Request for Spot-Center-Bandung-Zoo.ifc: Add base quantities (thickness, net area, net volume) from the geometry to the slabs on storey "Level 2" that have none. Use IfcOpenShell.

First a look at what the model holds.

```python
import ifcopenshell
import ifcopenshell.util.element
import ifcopenshell.util.unit

model = ifcopenshell.open("Spot-Center-Bandung-Zoo.ifc")
print(model.schema)
for unit_type in ("LENGTHUNIT", "AREAUNIT", "VOLUMEUNIT"):
    print(unit_type, ifcopenshell.util.unit.calculate_unit_scale(model, unit_type))
storey = next(s for s in model.by_type("IfcBuildingStorey") if s.Name == "Level 2")
slabs = [e for e in ifcopenshell.util.element.get_decomposition(storey) if e.is_a("IfcSlab")]
for e in sorted(slabs, key=lambda e: e.id()):
    print(e.id(), e.is_a(), e.Name, list(ifcopenshell.util.element.get_psets(e, qtos_only=True)), sep=" | ")
```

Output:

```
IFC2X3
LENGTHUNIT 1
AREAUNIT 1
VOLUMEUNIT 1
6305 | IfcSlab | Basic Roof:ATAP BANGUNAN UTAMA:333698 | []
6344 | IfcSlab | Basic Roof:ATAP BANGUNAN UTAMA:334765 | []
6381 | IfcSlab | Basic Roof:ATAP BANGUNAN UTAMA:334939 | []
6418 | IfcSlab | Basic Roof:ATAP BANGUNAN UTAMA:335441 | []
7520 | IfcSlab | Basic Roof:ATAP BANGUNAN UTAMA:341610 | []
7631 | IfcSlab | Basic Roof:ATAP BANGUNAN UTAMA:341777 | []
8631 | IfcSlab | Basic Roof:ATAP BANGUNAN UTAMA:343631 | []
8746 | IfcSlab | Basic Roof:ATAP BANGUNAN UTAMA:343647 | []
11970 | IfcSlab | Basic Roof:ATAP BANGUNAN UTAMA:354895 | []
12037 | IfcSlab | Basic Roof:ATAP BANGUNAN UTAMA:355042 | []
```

```python
import ifcopenshell
import ifcopenshell.api.pset
import ifcopenshell.geom
import ifcopenshell.util.element
import ifcopenshell.util.shape
import ifcopenshell.util.unit

model = ifcopenshell.open("Spot-Center-Bandung-Zoo.ifc")
unit_scale = ifcopenshell.util.unit.calculate_unit_scale(model)
area_scale = ifcopenshell.util.unit.calculate_unit_scale(model, "AREAUNIT")
volume_scale = ifcopenshell.util.unit.calculate_unit_scale(model, "VOLUMEUNIT")
settings = ifcopenshell.geom.settings()

storey = next(s for s in model.by_type("IfcBuildingStorey") if s.Name == "Level 2")
slabs = [e for e in ifcopenshell.util.element.get_decomposition(storey) if e.is_a("IfcSlab")]

for e in sorted(slabs, key=lambda e: e.id()):
    if ifcopenshell.util.element.get_psets(e, qtos_only=True, should_inherit=False):
        continue
    # Geometry comes back in metres, in the element's own axes.
    shape = ifcopenshell.geom.create_shape(settings, e)
    values = {
        "Width": ifcopenshell.util.shape.get_z(shape.geometry) / unit_scale,
        "NetArea": ifcopenshell.util.shape.get_footprint_area(shape.geometry) / area_scale,
        "NetVolume": ifcopenshell.util.shape.get_volume(shape.geometry) / volume_scale,
    }
    qto = ifcopenshell.api.pset.add_qto(model, product=e, name="BaseQuantities")
    ifcopenshell.api.pset.edit_qto(model, qto=qto, properties=values)
    print(e.id(), {k: round(v, 3) for k, v in values.items()})

model.write("Spot-Center-Bandung-Zoo_edited.ifc")
```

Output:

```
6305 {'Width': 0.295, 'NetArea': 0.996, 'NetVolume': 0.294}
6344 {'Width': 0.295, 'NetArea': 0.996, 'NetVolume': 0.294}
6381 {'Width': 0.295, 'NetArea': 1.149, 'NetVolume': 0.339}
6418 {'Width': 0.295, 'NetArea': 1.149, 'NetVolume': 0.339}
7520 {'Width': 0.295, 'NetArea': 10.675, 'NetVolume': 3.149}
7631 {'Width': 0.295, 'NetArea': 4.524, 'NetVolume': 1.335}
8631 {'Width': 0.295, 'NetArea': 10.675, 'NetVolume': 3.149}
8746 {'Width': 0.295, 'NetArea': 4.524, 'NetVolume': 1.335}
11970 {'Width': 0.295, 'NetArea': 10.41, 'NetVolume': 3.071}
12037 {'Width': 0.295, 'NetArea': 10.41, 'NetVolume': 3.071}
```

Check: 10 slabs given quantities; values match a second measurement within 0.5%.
